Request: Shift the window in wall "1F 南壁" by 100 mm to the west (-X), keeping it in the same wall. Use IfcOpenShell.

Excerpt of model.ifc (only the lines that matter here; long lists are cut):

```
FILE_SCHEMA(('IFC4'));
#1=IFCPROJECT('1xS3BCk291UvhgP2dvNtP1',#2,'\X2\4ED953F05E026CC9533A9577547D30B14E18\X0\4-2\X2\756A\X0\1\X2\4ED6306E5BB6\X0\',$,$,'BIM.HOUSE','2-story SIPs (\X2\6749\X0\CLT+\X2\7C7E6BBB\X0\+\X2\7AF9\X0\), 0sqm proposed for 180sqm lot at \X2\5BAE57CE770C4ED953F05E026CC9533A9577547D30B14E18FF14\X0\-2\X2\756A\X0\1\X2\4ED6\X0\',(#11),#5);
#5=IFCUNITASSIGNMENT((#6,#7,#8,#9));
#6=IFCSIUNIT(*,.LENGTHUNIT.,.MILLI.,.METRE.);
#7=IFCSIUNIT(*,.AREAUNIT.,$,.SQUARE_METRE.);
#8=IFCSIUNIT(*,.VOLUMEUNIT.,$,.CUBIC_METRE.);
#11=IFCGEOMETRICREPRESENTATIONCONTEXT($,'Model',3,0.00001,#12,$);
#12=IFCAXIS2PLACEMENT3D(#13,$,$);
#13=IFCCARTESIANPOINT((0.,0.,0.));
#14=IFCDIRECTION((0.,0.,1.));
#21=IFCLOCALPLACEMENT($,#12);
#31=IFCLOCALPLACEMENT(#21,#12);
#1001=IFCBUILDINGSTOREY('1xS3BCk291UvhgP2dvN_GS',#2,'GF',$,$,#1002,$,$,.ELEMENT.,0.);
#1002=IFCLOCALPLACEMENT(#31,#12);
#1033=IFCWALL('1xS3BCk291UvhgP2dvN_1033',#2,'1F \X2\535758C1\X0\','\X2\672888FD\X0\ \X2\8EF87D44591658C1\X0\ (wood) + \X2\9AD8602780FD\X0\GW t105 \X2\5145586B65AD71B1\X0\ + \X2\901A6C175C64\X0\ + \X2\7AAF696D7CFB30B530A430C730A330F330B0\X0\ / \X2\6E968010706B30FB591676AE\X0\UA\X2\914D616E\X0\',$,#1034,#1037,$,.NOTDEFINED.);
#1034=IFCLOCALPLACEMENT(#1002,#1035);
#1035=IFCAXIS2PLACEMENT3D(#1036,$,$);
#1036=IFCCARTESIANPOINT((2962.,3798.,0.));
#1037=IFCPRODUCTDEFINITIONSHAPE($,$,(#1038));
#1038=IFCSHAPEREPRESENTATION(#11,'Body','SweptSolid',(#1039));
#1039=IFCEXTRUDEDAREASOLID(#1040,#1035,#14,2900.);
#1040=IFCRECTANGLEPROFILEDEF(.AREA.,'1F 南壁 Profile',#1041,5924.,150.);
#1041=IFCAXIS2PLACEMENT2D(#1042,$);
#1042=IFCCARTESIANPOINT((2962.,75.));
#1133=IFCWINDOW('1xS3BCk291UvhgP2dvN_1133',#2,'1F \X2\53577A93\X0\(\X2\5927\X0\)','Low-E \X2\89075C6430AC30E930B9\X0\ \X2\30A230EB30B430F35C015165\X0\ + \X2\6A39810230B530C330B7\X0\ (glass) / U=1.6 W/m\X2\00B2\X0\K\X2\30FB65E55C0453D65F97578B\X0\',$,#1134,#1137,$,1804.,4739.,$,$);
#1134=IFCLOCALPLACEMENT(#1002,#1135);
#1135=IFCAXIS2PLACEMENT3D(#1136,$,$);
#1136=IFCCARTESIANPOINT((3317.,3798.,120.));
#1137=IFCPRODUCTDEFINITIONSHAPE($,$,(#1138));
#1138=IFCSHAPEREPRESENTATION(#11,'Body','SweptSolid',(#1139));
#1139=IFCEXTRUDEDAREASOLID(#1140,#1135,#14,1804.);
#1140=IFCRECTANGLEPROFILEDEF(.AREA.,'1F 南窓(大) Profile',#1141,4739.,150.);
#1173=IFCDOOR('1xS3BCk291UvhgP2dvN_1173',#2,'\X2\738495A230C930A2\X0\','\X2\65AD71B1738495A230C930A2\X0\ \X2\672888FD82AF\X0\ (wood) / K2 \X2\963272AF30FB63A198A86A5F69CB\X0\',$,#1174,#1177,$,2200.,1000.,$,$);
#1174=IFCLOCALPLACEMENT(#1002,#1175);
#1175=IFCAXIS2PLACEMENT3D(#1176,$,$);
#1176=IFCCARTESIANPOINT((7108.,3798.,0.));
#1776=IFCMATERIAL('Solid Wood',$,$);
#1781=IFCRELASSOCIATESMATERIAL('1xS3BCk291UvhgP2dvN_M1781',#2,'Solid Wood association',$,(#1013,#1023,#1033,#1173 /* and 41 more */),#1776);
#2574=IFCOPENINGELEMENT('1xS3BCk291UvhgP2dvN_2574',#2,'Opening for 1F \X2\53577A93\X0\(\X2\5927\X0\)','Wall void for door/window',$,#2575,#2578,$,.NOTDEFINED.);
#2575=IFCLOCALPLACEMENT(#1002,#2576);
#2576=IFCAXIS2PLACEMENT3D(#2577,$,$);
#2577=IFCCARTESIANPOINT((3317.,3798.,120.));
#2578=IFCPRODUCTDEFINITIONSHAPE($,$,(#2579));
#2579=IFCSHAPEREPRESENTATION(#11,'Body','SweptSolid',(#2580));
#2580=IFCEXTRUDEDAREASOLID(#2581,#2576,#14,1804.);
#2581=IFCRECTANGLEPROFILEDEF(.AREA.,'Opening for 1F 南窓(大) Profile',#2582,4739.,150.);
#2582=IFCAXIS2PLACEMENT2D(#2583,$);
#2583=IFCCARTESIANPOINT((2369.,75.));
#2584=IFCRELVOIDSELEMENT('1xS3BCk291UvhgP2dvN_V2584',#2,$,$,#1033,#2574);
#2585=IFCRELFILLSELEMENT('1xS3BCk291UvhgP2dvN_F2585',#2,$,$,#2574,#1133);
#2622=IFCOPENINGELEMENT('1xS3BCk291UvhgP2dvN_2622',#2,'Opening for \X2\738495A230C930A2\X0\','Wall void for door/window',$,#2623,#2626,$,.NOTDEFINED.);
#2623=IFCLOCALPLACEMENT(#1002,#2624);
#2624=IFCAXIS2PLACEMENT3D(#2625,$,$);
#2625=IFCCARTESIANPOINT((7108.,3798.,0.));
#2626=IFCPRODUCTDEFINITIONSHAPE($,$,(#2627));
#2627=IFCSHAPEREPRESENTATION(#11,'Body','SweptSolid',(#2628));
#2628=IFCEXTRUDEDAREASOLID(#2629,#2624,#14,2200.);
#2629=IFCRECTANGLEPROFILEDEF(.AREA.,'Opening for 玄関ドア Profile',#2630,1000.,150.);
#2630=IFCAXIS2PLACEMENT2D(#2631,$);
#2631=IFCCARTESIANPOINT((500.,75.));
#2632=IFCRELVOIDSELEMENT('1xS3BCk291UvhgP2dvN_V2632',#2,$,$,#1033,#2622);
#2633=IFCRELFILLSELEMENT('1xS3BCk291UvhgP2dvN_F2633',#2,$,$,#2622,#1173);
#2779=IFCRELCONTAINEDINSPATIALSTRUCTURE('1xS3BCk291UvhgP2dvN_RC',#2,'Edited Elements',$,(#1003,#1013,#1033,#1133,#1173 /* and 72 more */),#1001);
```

```python
import ifcopenshell
import ifcopenshell.api.geometry
import ifcopenshell.util.placement
import ifcopenshell.util.unit

model = ifcopenshell.open("model.ifc")
unit_scale = ifcopenshell.util.unit.calculate_unit_scale(model)

window = model.by_guid("1xS3BCk291UvhgP2dvN_1133")
opening = window.FillsVoids[0].RelatingOpeningElement
wall = opening.VoidsElements[0].RelatingBuildingElement

wall_matrix = ifcopenshell.util.placement.get_local_placement(wall.ObjectPlacement)
shift = wall_matrix[:3, 0] * -0.1 / unit_scale
before = ifcopenshell.util.placement.get_local_placement(window.ObjectPlacement)[:3, 3].copy()

# The window is not placed relative to its opening, so move both.
for product in (opening, window):
    matrix = ifcopenshell.util.placement.get_local_placement(product.ObjectPlacement)
    matrix[:3, 3] += shift
    ifcopenshell.api.geometry.edit_object_placement(model, product=product, matrix=matrix, is_si=False)

after = ifcopenshell.util.placement.get_local_placement(window.ObjectPlacement)[:3, 3]
print("window moved by", (after - before).round(3) + 0.0)

model.write("model_edited.ifc")
```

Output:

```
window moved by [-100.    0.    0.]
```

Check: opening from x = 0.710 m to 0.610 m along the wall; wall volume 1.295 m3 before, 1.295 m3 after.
